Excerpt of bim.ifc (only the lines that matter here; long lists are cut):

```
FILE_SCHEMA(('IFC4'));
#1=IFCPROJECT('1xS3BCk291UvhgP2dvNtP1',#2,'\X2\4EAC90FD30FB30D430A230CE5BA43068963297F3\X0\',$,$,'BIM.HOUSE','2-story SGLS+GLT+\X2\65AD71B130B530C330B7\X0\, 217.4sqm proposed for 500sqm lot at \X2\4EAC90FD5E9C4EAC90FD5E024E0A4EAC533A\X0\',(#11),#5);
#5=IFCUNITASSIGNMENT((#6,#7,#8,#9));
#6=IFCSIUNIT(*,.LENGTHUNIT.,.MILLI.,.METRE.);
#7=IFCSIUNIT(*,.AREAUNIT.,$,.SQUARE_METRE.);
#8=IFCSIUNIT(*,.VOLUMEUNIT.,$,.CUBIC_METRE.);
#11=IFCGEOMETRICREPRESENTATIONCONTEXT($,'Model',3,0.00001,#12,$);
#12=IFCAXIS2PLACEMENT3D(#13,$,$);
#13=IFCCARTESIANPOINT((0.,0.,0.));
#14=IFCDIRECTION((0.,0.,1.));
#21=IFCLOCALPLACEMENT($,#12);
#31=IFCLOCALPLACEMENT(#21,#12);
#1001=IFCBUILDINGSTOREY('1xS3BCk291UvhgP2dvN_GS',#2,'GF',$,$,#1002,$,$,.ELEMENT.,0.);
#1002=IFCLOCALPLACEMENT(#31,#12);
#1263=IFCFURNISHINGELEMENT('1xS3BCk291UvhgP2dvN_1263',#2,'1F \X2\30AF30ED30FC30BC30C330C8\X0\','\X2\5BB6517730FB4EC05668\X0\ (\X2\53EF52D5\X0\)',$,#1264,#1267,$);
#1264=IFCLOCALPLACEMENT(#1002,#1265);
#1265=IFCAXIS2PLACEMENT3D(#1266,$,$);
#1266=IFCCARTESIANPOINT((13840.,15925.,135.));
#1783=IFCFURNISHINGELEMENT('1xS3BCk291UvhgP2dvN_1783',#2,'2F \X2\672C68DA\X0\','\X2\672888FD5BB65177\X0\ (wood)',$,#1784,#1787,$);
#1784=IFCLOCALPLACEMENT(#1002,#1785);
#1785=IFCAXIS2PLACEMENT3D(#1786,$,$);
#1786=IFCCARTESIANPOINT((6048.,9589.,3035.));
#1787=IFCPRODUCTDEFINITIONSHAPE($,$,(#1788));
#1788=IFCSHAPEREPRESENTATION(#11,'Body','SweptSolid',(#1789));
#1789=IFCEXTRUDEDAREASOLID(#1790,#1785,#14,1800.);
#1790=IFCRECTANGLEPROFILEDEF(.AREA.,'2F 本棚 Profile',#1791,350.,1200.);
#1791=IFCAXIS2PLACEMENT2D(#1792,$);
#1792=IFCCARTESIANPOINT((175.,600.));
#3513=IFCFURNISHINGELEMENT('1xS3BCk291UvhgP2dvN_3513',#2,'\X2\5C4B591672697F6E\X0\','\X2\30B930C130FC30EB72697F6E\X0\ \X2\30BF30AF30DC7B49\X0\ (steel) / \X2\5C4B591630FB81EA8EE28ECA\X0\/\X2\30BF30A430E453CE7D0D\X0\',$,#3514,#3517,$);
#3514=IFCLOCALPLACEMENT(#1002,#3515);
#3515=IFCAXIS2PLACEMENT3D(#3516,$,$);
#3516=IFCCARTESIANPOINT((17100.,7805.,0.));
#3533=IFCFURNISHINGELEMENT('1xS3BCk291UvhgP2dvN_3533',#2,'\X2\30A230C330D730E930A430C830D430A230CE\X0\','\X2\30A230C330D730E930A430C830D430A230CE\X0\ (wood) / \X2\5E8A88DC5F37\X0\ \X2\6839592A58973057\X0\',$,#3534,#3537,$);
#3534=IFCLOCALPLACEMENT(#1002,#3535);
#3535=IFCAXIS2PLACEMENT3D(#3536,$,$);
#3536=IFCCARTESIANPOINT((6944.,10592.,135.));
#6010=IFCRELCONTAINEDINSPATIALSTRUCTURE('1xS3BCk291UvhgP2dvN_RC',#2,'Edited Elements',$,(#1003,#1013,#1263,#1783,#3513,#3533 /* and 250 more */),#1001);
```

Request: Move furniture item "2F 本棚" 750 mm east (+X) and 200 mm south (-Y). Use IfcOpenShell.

```python
import ifcopenshell
import ifcopenshell.api.geometry
import ifcopenshell.util.placement
import ifcopenshell.util.unit

model = ifcopenshell.open("bim.ifc")
unit_scale = ifcopenshell.util.unit.calculate_unit_scale(model)

item = model.by_guid("1xS3BCk291UvhgP2dvN_1783")
matrix = ifcopenshell.util.placement.get_local_placement(item.ObjectPlacement)
matrix[0, 3] += 0.75 / unit_scale
matrix[1, 3] -= 0.2 / unit_scale
ifcopenshell.api.geometry.edit_object_placement(model, product=item, matrix=matrix, is_si=False)

print(ifcopenshell.util.placement.get_local_placement(item.ObjectPlacement).round(3) + 0.0)

model.write("bim_updated.ifc")
```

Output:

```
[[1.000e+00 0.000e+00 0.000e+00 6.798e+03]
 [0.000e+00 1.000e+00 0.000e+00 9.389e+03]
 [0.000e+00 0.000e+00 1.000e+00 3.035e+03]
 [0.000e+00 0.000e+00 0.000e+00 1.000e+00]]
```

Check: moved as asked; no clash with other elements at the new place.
